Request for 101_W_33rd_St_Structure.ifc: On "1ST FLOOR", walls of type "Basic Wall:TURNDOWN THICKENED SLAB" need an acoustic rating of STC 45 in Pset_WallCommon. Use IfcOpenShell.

First a look at what the model holds.

```python
import ifcopenshell
import ifcopenshell.util.element

model = ifcopenshell.open("101_W_33rd_St_Structure.ifc")
print(model.schema)
storey = next(s for s in model.by_type("IfcBuildingStorey") if s.Name == "1ST FLOOR")
walls = [e for e in ifcopenshell.util.element.get_decomposition(storey) if e.is_a("IfcWall")]
seen = {}
for e in walls:
    element_type = ifcopenshell.util.element.get_type(e)
    key = (element_type.Name if element_type != e and element_type else None, ifcopenshell.util.element.get_pset(e, "Pset_WallCommon", "AcousticRating"))
    seen[key] = seen.get(key, 0) + 1
for (name, value), count in sorted(seen.items(), key=str):
    print(count, "x", name, "|", value)
```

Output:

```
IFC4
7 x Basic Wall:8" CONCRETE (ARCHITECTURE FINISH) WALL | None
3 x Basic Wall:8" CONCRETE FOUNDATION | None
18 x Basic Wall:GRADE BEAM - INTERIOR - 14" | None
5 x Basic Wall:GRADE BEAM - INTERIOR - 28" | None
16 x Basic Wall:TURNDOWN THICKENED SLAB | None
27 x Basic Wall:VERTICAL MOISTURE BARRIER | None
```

```python
import ifcopenshell
import ifcopenshell.api.pset
import ifcopenshell.util.element

model = ifcopenshell.open("101_W_33rd_St_Structure.ifc")

storey = next(s for s in model.by_type("IfcBuildingStorey") if s.Name == "1ST FLOOR")
walls = [e for e in ifcopenshell.util.element.get_decomposition(storey) if e.is_a("IfcWall")]

count = 0
for e in walls:
    element_type = ifcopenshell.util.element.get_type(e)
    if element_type in (None, e) or element_type.Name != "Basic Wall:TURNDOWN THICKENED SLAB":
        continue
    # add_pset returns the element's existing set when there is one.
    pset = ifcopenshell.api.pset.add_pset(model, product=e, name="Pset_WallCommon")
    ifcopenshell.api.pset.edit_pset(model, pset=pset, properties={"AcousticRating": "STC 45"})
    count += 1

print(count, "walls updated")

model.write("101_W_33rd_St_Structure-out.ifc")
```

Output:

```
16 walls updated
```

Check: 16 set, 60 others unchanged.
